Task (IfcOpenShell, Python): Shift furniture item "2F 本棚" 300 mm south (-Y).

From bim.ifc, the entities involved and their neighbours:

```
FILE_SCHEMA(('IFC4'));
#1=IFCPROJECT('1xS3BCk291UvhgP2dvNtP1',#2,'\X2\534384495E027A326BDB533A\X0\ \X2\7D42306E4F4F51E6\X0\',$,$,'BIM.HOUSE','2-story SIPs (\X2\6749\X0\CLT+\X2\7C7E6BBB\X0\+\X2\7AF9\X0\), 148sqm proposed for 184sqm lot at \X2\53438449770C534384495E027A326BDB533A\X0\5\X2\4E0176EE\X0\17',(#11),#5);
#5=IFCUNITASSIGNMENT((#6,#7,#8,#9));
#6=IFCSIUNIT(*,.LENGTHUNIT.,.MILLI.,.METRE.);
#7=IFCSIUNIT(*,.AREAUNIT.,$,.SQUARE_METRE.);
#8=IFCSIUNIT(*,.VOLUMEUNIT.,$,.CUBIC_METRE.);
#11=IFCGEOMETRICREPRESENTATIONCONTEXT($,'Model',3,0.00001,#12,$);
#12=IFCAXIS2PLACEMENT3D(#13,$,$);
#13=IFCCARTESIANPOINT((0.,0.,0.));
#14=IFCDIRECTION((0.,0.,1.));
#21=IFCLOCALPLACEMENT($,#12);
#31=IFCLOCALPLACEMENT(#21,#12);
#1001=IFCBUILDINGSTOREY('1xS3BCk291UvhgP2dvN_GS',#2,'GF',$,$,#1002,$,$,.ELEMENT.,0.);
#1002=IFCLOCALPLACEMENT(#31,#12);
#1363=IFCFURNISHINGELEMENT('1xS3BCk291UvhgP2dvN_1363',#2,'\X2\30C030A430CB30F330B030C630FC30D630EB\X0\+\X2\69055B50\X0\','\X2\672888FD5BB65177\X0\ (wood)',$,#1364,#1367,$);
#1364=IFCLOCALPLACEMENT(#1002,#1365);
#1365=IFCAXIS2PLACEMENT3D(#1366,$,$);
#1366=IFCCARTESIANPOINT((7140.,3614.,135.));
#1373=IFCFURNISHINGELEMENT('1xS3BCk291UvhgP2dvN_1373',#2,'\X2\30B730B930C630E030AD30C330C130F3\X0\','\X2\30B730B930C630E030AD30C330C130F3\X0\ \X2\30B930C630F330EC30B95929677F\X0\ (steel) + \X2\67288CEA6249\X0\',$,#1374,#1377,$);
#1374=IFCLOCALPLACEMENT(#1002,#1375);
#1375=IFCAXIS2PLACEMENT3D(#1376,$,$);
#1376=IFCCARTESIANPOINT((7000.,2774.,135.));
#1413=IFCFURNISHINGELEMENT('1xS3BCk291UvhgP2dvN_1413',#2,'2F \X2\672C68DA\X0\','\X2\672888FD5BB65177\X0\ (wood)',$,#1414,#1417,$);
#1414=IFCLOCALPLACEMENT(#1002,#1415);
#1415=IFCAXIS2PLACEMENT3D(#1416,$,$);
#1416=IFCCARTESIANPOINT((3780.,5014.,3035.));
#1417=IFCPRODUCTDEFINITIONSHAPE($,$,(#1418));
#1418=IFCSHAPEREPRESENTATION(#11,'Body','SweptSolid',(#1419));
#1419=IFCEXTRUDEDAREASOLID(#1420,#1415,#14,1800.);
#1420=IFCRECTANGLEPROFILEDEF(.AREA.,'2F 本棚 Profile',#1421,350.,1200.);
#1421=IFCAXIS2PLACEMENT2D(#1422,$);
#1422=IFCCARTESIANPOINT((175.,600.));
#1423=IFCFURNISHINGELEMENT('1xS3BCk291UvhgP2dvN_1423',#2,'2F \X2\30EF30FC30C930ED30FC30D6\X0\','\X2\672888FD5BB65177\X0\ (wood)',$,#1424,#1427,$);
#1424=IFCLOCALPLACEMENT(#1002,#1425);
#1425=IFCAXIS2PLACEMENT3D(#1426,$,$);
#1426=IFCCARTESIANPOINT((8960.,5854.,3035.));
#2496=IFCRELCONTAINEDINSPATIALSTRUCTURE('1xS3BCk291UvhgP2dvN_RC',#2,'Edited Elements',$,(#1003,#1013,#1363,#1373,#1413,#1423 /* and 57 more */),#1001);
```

```python
import ifcopenshell
import ifcopenshell.api.geometry
import ifcopenshell.util.placement
import ifcopenshell.util.unit

model = ifcopenshell.open("bim.ifc")
unit_scale = ifcopenshell.util.unit.calculate_unit_scale(model)

item = model.by_guid("1xS3BCk291UvhgP2dvN_1413")
matrix = ifcopenshell.util.placement.get_local_placement(item.ObjectPlacement)
matrix[1, 3] -= 0.3 / unit_scale
ifcopenshell.api.geometry.edit_object_placement(model, product=item, matrix=matrix, is_si=False)

print(ifcopenshell.util.placement.get_local_placement(item.ObjectPlacement).round(3) + 0.0)

model.write("bim_updated.ifc")
```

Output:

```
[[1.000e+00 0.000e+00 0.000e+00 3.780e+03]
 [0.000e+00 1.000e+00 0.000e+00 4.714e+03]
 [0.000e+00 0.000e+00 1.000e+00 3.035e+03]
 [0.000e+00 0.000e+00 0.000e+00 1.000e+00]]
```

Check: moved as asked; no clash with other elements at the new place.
